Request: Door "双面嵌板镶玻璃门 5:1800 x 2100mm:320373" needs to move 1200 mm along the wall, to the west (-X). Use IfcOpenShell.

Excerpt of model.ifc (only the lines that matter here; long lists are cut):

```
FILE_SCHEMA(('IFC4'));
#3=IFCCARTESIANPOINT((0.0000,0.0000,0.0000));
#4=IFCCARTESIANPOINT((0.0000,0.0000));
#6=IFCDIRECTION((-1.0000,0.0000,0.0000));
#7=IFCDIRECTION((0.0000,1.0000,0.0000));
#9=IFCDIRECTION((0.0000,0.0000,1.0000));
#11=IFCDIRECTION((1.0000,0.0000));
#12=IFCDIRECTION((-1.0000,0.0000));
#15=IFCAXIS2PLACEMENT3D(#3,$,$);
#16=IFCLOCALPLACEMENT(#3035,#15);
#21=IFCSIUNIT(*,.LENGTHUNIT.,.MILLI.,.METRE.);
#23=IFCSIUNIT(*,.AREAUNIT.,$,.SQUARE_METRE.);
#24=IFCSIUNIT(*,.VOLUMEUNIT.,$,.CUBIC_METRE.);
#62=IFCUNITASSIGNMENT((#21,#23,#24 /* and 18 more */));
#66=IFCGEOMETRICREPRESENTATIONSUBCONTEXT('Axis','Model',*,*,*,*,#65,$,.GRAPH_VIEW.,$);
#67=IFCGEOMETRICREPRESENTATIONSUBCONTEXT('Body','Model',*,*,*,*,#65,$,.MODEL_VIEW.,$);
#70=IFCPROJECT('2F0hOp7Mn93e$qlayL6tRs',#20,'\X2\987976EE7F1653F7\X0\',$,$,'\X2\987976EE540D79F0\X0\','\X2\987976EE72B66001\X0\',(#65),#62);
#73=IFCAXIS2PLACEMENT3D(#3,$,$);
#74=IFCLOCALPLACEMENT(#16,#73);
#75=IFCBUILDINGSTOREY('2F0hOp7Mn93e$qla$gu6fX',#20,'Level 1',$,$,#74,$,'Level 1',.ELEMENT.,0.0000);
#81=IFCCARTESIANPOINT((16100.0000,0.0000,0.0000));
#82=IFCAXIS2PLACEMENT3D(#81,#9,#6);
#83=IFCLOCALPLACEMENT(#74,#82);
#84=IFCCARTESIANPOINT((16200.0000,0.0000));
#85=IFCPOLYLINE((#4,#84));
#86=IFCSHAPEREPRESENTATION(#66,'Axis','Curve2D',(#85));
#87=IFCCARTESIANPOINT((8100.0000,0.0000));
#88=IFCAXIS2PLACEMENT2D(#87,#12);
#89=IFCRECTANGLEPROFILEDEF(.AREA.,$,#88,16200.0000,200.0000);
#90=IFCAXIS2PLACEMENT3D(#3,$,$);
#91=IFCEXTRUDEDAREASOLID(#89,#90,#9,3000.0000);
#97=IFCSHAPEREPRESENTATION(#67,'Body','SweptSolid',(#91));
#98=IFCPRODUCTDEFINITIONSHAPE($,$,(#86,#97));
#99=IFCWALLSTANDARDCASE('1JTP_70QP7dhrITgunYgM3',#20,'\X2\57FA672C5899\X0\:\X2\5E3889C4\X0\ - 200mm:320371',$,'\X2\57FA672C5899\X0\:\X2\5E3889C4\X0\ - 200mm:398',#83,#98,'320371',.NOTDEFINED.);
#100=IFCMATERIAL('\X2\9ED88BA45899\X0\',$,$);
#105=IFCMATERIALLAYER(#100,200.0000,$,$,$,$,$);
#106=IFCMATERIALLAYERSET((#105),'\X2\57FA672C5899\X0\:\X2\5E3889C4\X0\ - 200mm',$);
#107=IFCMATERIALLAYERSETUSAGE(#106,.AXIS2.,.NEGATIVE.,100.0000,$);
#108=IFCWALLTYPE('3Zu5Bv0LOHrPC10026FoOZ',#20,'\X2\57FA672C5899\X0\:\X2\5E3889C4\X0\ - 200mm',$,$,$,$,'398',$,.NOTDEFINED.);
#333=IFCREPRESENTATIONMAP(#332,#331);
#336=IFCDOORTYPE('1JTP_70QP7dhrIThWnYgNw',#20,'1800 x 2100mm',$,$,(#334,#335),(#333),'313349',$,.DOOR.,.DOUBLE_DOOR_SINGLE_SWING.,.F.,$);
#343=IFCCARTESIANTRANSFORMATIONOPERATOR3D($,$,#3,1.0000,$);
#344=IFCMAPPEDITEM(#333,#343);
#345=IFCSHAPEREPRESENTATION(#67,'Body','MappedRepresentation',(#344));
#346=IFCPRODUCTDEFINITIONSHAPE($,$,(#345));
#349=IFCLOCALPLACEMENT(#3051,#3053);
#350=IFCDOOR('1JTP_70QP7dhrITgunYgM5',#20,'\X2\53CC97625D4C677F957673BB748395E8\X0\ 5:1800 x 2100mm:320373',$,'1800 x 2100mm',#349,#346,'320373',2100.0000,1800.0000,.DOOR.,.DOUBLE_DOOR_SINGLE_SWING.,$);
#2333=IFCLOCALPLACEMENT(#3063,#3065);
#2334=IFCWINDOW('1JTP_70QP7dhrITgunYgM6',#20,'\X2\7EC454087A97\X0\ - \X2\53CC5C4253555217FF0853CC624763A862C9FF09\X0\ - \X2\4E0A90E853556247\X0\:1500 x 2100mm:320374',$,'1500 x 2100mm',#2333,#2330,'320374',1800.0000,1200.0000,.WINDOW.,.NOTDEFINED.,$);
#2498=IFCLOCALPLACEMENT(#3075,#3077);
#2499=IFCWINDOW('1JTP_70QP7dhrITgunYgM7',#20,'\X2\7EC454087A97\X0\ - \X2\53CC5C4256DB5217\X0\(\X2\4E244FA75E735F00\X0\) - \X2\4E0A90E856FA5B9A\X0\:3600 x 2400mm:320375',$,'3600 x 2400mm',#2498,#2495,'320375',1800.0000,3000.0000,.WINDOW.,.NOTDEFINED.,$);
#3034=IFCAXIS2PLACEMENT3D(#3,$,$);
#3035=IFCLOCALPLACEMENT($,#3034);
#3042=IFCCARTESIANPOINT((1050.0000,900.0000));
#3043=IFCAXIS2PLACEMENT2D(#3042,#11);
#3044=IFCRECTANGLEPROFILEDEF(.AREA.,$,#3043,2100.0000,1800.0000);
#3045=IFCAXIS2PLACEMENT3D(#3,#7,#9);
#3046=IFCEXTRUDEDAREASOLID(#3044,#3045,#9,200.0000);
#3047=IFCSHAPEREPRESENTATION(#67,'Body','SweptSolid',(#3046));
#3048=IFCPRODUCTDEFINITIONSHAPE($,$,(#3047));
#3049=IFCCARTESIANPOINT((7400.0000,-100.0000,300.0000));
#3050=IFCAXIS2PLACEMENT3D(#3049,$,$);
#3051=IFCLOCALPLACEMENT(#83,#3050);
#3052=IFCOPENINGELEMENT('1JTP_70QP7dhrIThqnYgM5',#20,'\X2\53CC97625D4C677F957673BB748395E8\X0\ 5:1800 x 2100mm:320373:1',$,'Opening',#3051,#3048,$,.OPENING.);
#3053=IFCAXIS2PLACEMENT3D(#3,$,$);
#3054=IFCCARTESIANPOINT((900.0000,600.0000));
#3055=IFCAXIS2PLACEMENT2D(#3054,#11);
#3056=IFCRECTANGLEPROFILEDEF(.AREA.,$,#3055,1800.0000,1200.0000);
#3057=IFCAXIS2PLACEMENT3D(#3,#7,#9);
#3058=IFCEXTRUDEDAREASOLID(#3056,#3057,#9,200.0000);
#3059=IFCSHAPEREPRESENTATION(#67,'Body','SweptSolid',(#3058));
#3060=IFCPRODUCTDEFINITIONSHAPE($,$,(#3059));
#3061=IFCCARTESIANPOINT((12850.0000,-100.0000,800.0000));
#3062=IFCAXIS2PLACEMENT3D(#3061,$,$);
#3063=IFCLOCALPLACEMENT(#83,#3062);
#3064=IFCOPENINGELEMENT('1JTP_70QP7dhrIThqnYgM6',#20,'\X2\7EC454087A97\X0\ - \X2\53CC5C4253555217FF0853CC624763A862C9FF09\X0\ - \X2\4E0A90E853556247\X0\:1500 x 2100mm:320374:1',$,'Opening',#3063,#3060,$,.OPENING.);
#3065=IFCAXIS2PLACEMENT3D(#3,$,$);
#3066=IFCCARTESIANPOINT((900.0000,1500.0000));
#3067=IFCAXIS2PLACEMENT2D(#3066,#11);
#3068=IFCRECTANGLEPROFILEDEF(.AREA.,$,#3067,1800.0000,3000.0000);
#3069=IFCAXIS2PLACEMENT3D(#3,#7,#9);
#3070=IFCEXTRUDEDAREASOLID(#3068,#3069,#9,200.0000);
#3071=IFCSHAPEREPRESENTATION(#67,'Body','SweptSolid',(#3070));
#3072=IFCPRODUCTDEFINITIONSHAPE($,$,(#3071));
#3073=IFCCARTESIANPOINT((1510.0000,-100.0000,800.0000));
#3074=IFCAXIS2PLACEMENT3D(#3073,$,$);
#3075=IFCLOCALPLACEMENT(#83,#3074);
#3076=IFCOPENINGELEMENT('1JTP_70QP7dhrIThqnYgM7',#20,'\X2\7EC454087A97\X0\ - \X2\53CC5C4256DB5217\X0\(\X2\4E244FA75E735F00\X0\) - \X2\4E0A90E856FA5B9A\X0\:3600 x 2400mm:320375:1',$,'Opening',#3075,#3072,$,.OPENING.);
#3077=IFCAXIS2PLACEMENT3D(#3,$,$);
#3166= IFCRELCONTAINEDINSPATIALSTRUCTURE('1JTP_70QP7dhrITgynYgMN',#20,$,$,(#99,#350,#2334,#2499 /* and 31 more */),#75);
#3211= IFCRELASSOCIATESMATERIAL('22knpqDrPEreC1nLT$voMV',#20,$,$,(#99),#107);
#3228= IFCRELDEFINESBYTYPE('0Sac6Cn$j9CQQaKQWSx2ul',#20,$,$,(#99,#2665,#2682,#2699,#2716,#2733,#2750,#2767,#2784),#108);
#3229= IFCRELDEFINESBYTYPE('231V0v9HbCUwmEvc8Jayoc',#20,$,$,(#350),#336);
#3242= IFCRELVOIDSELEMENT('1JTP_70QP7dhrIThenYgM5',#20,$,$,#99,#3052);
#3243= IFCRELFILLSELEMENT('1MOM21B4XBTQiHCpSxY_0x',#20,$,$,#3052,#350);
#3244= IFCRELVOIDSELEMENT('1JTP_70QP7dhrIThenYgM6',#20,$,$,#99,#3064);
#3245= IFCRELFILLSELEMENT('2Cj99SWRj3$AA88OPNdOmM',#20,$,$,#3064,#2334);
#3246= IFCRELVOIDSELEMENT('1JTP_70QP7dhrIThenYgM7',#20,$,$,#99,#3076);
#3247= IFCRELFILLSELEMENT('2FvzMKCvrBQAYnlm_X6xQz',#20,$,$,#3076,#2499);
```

```python
import ifcopenshell
import ifcopenshell.api.geometry
import ifcopenshell.util.placement

model = ifcopenshell.open("model.ifc")

door = model.by_guid("1JTP_70QP7dhrITgunYgM5")
opening = door.FillsVoids[0].RelatingOpeningElement
wall = opening.VoidsElements[0].RelatingBuildingElement

wall_matrix = ifcopenshell.util.placement.get_local_placement(wall.ObjectPlacement)
shift = wall_matrix[:3, 0] * 1200.0
before = ifcopenshell.util.placement.get_local_placement(door.ObjectPlacement)[:3, 3].copy()

# The door is placed relative to its opening, so it follows when the opening moves.
matrix = ifcopenshell.util.placement.get_local_placement(opening.ObjectPlacement)
matrix[:3, 3] += shift
ifcopenshell.api.geometry.edit_object_placement(
    model, product=opening, matrix=matrix, is_si=False, should_transform_children=True
)

after = ifcopenshell.util.placement.get_local_placement(door.ObjectPlacement)[:3, 3]
print("door moved by", (after - before).round(3) + 0.0)

model.write("model_rev.ifc")
```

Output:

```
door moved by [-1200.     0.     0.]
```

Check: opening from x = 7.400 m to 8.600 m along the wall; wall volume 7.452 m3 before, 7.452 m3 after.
